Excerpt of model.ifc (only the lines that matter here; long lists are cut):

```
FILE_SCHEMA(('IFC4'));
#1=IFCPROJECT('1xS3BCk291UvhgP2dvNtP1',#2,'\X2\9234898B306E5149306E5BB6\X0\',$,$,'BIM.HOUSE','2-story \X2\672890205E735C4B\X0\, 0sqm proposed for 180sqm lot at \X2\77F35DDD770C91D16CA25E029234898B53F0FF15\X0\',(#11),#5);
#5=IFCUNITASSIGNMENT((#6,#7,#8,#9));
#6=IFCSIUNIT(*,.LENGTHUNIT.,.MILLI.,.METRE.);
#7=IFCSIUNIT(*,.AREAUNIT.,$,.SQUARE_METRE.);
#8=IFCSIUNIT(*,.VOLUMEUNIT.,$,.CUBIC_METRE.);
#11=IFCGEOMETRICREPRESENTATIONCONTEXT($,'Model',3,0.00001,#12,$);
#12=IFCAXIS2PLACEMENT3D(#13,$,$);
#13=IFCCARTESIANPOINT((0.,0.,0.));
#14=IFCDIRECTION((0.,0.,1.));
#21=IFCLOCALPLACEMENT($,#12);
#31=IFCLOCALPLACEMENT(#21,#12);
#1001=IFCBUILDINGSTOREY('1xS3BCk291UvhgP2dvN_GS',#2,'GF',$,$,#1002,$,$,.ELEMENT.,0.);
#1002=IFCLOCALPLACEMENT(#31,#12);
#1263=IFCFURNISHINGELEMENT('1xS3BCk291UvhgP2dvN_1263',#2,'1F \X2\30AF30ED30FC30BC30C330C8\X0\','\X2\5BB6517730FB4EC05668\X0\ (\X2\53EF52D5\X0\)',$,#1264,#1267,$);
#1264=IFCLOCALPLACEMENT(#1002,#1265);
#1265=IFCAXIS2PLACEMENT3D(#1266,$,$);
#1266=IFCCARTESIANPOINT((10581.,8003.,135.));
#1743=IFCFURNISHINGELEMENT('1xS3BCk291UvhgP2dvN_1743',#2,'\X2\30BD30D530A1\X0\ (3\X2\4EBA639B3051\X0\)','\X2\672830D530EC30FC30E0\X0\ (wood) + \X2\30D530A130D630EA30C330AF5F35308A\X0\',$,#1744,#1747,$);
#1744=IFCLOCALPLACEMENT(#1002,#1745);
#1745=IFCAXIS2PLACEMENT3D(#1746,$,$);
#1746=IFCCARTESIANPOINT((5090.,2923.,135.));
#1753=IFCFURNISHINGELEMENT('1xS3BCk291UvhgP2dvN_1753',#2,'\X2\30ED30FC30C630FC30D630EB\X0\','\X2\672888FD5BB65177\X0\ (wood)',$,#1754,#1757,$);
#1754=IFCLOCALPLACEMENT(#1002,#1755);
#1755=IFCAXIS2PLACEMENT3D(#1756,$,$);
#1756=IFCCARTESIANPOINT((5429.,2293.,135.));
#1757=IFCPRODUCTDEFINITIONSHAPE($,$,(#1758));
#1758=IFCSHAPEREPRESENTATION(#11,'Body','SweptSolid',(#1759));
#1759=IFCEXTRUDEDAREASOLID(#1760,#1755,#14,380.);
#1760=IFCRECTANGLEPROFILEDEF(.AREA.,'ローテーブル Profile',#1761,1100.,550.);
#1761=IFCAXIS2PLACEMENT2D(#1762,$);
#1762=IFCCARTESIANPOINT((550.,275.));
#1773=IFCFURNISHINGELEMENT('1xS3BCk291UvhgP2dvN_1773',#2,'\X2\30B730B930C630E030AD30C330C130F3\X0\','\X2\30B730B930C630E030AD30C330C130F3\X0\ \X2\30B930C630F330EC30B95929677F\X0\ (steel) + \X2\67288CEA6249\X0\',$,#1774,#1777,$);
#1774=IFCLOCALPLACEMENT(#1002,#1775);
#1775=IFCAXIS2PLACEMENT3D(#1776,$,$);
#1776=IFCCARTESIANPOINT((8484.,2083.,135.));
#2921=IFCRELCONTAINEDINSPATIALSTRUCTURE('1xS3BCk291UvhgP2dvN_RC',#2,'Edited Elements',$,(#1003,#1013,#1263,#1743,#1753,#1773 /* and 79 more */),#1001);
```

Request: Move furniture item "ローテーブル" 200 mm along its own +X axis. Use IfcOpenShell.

```python
import ifcopenshell
import ifcopenshell.api.geometry
import ifcopenshell.util.placement
import ifcopenshell.util.unit

model = ifcopenshell.open("model.ifc")
unit_scale = ifcopenshell.util.unit.calculate_unit_scale(model)

item = model.by_guid("1xS3BCk291UvhgP2dvN_1753")
matrix = ifcopenshell.util.placement.get_local_placement(item.ObjectPlacement)
matrix[:3, 3] += matrix[:3, 0] * 0.2 / unit_scale
ifcopenshell.api.geometry.edit_object_placement(model, product=item, matrix=matrix, is_si=False)

print(ifcopenshell.util.placement.get_local_placement(item.ObjectPlacement).round(3) + 0.0)

model.write("model_v2.ifc")
```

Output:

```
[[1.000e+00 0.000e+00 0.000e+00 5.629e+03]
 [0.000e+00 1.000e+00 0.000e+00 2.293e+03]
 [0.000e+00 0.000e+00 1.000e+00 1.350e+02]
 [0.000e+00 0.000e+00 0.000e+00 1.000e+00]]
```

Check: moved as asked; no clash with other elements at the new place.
